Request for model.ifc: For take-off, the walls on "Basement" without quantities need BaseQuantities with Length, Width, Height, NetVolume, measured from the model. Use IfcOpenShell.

First a look at what the model holds.

```python
import ifcopenshell
import ifcopenshell.util.element
import ifcopenshell.util.unit

model = ifcopenshell.open("model.ifc")
print(model.schema)
for unit_type in ("LENGTHUNIT", "AREAUNIT", "VOLUMEUNIT"):
    print(unit_type, ifcopenshell.util.unit.calculate_unit_scale(model, unit_type))
storey = next(s for s in model.by_type("IfcBuildingStorey") if s.Name == "Basement")
walls = [e for e in ifcopenshell.util.element.get_decomposition(storey) if e.is_a("IfcWall")]
for e in sorted(walls, key=lambda e: e.id()):
    print(e.id(), e.is_a(), e.Name, list(ifcopenshell.util.element.get_psets(e, qtos_only=True)), sep=" | ")
```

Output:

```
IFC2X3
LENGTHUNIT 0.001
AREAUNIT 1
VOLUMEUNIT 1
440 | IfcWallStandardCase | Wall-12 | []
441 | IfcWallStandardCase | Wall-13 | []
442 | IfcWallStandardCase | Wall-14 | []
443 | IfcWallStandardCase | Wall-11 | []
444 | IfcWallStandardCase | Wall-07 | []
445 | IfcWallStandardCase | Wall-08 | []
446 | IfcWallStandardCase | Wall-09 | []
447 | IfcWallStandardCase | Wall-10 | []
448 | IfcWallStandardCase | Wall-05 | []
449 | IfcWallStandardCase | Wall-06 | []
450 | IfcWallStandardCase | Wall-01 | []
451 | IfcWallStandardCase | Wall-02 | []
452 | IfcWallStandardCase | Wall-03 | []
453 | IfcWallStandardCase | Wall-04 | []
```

```python
import ifcopenshell
import ifcopenshell.api.pset
import ifcopenshell.geom
import ifcopenshell.util.element
import ifcopenshell.util.shape
import ifcopenshell.util.unit

model = ifcopenshell.open("model.ifc")
unit_scale = ifcopenshell.util.unit.calculate_unit_scale(model)
volume_scale = ifcopenshell.util.unit.calculate_unit_scale(model, "VOLUMEUNIT")
settings = ifcopenshell.geom.settings()

storey = next(s for s in model.by_type("IfcBuildingStorey") if s.Name == "Basement")
walls = [e for e in ifcopenshell.util.element.get_decomposition(storey) if e.is_a("IfcWall")]

for e in sorted(walls, key=lambda e: e.id()):
    if ifcopenshell.util.element.get_psets(e, qtos_only=True, should_inherit=False):
        continue
    # Geometry comes back in metres, in the element's own axes.
    shape = ifcopenshell.geom.create_shape(settings, e)
    values = {
        "Length": ifcopenshell.util.shape.get_x(shape.geometry) / unit_scale,
        "Width": ifcopenshell.util.shape.get_y(shape.geometry) / unit_scale,
        "Height": ifcopenshell.util.shape.get_z(shape.geometry) / unit_scale,
        "NetVolume": ifcopenshell.util.shape.get_volume(shape.geometry) / volume_scale,
    }
    qto = ifcopenshell.api.pset.add_qto(model, product=e, name="BaseQuantities")
    ifcopenshell.api.pset.edit_qto(model, qto=qto, properties=values)
    print(e.id(), {k: round(v, 3) for k, v in values.items()})

model.write("model_v2.ifc")
```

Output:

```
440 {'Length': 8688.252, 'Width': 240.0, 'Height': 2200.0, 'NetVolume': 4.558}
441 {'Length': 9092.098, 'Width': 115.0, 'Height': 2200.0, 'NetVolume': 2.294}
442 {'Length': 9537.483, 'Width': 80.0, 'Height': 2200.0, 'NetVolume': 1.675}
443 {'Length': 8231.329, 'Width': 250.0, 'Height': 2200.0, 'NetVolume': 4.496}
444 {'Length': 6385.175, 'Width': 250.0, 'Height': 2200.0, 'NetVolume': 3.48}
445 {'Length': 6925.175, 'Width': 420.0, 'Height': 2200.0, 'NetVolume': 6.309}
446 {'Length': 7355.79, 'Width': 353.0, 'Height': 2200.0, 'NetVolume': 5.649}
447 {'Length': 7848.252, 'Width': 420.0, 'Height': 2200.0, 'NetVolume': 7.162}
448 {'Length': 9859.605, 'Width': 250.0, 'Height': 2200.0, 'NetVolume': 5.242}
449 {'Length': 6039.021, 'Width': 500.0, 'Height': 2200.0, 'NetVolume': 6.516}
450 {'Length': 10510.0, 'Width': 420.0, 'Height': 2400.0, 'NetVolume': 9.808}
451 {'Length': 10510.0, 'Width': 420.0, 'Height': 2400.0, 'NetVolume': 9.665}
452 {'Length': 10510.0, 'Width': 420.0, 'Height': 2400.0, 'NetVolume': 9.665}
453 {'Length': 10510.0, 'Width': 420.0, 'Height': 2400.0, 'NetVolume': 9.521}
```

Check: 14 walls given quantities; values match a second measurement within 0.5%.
